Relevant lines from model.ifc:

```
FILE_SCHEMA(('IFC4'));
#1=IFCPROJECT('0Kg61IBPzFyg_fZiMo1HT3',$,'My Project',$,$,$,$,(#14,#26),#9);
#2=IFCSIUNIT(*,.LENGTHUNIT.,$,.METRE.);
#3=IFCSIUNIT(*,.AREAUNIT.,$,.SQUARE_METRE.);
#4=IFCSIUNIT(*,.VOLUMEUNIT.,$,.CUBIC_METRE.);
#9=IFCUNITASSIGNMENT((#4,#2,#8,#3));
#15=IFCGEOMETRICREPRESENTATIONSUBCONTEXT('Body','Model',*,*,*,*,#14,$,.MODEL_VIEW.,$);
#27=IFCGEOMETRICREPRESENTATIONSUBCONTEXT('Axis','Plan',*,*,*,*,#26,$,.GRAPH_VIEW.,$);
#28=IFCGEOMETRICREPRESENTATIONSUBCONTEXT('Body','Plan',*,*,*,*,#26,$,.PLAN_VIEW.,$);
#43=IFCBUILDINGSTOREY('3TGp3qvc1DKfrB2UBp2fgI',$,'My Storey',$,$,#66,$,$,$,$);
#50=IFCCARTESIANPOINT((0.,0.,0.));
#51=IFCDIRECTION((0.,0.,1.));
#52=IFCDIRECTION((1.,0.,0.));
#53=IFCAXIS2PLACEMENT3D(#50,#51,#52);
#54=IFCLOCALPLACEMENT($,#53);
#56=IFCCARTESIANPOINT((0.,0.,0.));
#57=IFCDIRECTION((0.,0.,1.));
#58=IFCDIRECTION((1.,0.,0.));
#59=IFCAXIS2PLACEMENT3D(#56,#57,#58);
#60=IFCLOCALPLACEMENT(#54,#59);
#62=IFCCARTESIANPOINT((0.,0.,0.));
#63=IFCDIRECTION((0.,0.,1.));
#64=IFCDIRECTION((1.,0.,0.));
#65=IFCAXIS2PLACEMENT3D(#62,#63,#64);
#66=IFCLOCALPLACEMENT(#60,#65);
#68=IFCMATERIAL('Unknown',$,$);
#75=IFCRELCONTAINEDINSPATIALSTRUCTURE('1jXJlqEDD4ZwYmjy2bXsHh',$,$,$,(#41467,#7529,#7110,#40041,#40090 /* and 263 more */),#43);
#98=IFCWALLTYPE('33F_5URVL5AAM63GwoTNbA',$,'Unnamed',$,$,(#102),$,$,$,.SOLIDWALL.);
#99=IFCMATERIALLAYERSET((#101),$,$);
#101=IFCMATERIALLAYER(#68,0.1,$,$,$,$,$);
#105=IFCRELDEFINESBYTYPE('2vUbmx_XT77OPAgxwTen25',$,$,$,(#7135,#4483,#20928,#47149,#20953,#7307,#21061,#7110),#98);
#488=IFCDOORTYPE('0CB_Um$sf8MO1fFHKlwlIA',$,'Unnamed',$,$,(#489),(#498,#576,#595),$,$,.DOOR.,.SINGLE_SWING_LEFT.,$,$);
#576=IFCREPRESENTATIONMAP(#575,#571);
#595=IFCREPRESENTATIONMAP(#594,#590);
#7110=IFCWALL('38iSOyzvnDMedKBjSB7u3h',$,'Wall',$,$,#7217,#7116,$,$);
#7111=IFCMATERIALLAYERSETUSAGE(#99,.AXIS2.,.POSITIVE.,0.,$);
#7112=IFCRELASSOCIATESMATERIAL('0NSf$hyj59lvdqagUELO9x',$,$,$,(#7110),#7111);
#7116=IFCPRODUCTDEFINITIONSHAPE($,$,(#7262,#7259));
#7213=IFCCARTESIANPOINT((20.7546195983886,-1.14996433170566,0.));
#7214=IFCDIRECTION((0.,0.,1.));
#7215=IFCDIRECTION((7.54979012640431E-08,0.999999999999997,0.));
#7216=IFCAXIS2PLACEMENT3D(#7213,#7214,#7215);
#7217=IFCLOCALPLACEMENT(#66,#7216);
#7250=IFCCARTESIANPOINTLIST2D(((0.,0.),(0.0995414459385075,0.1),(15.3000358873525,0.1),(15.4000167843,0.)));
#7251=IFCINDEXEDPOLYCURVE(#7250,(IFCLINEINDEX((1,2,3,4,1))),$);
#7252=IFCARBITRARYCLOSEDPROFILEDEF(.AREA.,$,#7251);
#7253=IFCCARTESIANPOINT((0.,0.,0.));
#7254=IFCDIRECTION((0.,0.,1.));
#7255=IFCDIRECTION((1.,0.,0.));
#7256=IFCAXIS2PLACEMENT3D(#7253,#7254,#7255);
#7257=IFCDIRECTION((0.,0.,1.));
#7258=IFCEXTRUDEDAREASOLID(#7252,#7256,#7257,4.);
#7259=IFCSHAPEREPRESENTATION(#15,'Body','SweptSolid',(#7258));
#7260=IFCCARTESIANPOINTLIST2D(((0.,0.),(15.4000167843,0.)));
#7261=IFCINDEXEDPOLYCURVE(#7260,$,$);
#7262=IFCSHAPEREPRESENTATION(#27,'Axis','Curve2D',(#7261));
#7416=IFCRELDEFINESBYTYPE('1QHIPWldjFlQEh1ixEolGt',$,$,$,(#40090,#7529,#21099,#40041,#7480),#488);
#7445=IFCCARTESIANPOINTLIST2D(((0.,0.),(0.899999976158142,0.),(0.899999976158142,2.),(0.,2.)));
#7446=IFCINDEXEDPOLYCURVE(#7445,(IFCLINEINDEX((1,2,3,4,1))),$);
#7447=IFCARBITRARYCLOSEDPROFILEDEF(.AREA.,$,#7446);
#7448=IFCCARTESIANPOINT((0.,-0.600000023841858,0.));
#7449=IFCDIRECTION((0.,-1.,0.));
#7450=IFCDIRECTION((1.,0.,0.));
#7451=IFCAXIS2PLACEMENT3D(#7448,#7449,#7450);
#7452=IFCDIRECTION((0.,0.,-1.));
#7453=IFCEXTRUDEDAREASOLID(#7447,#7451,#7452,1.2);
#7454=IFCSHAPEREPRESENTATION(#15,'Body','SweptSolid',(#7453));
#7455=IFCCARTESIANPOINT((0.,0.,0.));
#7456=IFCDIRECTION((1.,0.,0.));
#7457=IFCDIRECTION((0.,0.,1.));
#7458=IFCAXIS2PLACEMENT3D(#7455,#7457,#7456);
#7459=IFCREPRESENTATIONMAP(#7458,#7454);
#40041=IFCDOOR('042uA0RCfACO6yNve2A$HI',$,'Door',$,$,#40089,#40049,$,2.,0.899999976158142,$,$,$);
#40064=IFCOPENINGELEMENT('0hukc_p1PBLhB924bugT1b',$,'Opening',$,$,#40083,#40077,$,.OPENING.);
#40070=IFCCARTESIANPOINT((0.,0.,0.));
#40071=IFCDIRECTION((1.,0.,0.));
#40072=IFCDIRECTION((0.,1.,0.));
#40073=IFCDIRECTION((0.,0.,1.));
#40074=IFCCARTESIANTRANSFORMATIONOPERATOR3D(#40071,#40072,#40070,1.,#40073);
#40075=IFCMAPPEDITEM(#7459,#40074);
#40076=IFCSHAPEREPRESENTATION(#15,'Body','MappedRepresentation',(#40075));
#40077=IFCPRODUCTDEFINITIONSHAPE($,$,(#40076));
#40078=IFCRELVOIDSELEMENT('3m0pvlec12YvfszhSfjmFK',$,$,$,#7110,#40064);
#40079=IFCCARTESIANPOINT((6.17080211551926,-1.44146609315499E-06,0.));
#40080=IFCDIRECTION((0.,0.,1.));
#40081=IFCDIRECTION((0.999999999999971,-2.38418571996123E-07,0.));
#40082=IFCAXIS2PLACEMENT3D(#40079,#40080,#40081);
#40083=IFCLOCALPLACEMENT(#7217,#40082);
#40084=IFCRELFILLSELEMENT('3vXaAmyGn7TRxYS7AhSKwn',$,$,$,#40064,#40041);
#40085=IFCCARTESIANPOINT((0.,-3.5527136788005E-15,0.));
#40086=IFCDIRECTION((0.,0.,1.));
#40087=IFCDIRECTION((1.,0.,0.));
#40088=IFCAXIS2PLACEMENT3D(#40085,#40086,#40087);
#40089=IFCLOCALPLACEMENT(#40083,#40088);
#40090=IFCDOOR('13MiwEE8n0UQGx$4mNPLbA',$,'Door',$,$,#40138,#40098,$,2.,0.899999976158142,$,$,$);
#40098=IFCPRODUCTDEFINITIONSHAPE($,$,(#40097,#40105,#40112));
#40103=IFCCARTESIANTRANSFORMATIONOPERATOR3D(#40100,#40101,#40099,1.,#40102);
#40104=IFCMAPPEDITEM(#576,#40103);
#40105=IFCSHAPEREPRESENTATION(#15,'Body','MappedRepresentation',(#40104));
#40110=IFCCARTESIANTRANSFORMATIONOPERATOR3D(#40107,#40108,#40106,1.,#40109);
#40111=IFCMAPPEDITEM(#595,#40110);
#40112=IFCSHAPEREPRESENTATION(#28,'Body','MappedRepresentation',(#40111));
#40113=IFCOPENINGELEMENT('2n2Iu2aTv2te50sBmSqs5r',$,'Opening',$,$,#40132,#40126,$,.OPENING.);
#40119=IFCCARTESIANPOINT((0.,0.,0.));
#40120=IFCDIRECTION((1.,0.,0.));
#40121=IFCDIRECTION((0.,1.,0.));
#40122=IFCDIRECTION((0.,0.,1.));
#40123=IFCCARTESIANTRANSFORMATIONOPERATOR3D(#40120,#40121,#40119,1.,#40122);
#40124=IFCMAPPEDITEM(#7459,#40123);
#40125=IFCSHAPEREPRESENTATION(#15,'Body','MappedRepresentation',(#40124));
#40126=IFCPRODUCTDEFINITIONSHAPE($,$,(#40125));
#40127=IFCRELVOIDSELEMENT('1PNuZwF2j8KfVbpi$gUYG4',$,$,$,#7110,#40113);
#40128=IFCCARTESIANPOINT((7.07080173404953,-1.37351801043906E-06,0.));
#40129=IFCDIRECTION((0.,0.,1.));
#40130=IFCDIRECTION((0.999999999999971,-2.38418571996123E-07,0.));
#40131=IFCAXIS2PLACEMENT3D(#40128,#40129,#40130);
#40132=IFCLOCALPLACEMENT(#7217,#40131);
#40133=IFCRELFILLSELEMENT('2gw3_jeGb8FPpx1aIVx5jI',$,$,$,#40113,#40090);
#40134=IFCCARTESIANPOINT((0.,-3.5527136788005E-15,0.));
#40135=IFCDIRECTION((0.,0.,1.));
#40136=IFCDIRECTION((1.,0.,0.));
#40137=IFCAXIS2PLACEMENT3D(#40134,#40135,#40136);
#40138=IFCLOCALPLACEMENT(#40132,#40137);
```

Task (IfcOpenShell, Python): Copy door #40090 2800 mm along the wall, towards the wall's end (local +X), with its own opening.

```python
import ifcopenshell
import ifcopenshell.api.feature
import ifcopenshell.api.geometry
import ifcopenshell.api.root
import ifcopenshell.geom
import ifcopenshell.util.element
import ifcopenshell.util.placement
import ifcopenshell.util.shape
import ifcopenshell.util.unit

model = ifcopenshell.open("model.ifc")
unit_scale = ifcopenshell.util.unit.calculate_unit_scale(model)
settings = ifcopenshell.geom.settings()


def volume(element):
    """Net volume in cubic metres, openings subtracted."""
    shape = ifcopenshell.geom.create_shape(settings, element)
    return ifcopenshell.util.shape.get_volume(shape.geometry)


door = model.by_guid("13MiwEE8n0UQGx$4mNPLbA")
opening = door.FillsVoids[0].RelatingOpeningElement
wall = opening.VoidsElements[0].RelatingBuildingElement
before = volume(wall)
shift = ifcopenshell.util.placement.get_local_placement(wall.ObjectPlacement)[:3, 0] * 2.8 / unit_scale

# copy_class copies the void relationship, type, container and properties, but no geometry.
new_opening = ifcopenshell.api.root.copy_class(model, product=opening)
new_opening.Representation = ifcopenshell.util.element.copy_deep(
    model, opening.Representation, exclude=["IfcGeometricRepresentationContext", "IfcRepresentationMap"]
)
new_door = ifcopenshell.api.root.copy_class(model, product=door)
new_door.Representation = ifcopenshell.util.element.copy_deep(
    model, door.Representation, exclude=["IfcGeometricRepresentationContext", "IfcRepresentationMap"]
)
ifcopenshell.api.feature.add_filling(model, opening=new_opening, element=new_door)

for old, new in ((opening, new_opening), (door, new_door)):
    matrix = ifcopenshell.util.placement.get_local_placement(old.ObjectPlacement)
    matrix[:3, 3] += shift
    ifcopenshell.api.geometry.edit_object_placement(model, product=new, matrix=matrix, is_si=False)

after = volume(wall)

print(f"wall volume {before:.3f} -> {after:.3f} m3")

model.write("model_v2.ifc")
```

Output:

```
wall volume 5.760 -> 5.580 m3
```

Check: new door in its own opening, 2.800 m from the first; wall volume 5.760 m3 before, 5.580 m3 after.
